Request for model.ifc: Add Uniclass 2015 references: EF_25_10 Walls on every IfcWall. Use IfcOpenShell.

First a look at what the model holds.

```python
import ifcopenshell

model = ifcopenshell.open("model.ifc")
print(model.schema)
print("classifications:", [c.Name for c in model.by_type("IfcClassification")])
for ifc_class in ("IfcDoor", "IfcRoof", "IfcStair", "IfcWall", "IfcWindow"):
    print(ifc_class, len(model.by_type(ifc_class)))
```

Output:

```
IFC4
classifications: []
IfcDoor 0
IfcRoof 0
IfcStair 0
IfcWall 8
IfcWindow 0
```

```python
import ifcopenshell
import ifcopenshell.api.classification

model = ifcopenshell.open("model.ifc")

system = ifcopenshell.api.classification.add_classification(model, classification="Uniclass 2015")

codes = {
    "IfcWall": ("EF_25_10", "Walls"),
}
for ifc_class, (code, name) in codes.items():
    products = model.by_type(ifc_class)
    ifcopenshell.api.classification.add_reference(
        model, products=products, classification=system, identification=code, name=name
    )
    print(code, len(products))

model.write("model_v2.ifc")
```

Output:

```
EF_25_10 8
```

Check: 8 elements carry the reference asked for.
